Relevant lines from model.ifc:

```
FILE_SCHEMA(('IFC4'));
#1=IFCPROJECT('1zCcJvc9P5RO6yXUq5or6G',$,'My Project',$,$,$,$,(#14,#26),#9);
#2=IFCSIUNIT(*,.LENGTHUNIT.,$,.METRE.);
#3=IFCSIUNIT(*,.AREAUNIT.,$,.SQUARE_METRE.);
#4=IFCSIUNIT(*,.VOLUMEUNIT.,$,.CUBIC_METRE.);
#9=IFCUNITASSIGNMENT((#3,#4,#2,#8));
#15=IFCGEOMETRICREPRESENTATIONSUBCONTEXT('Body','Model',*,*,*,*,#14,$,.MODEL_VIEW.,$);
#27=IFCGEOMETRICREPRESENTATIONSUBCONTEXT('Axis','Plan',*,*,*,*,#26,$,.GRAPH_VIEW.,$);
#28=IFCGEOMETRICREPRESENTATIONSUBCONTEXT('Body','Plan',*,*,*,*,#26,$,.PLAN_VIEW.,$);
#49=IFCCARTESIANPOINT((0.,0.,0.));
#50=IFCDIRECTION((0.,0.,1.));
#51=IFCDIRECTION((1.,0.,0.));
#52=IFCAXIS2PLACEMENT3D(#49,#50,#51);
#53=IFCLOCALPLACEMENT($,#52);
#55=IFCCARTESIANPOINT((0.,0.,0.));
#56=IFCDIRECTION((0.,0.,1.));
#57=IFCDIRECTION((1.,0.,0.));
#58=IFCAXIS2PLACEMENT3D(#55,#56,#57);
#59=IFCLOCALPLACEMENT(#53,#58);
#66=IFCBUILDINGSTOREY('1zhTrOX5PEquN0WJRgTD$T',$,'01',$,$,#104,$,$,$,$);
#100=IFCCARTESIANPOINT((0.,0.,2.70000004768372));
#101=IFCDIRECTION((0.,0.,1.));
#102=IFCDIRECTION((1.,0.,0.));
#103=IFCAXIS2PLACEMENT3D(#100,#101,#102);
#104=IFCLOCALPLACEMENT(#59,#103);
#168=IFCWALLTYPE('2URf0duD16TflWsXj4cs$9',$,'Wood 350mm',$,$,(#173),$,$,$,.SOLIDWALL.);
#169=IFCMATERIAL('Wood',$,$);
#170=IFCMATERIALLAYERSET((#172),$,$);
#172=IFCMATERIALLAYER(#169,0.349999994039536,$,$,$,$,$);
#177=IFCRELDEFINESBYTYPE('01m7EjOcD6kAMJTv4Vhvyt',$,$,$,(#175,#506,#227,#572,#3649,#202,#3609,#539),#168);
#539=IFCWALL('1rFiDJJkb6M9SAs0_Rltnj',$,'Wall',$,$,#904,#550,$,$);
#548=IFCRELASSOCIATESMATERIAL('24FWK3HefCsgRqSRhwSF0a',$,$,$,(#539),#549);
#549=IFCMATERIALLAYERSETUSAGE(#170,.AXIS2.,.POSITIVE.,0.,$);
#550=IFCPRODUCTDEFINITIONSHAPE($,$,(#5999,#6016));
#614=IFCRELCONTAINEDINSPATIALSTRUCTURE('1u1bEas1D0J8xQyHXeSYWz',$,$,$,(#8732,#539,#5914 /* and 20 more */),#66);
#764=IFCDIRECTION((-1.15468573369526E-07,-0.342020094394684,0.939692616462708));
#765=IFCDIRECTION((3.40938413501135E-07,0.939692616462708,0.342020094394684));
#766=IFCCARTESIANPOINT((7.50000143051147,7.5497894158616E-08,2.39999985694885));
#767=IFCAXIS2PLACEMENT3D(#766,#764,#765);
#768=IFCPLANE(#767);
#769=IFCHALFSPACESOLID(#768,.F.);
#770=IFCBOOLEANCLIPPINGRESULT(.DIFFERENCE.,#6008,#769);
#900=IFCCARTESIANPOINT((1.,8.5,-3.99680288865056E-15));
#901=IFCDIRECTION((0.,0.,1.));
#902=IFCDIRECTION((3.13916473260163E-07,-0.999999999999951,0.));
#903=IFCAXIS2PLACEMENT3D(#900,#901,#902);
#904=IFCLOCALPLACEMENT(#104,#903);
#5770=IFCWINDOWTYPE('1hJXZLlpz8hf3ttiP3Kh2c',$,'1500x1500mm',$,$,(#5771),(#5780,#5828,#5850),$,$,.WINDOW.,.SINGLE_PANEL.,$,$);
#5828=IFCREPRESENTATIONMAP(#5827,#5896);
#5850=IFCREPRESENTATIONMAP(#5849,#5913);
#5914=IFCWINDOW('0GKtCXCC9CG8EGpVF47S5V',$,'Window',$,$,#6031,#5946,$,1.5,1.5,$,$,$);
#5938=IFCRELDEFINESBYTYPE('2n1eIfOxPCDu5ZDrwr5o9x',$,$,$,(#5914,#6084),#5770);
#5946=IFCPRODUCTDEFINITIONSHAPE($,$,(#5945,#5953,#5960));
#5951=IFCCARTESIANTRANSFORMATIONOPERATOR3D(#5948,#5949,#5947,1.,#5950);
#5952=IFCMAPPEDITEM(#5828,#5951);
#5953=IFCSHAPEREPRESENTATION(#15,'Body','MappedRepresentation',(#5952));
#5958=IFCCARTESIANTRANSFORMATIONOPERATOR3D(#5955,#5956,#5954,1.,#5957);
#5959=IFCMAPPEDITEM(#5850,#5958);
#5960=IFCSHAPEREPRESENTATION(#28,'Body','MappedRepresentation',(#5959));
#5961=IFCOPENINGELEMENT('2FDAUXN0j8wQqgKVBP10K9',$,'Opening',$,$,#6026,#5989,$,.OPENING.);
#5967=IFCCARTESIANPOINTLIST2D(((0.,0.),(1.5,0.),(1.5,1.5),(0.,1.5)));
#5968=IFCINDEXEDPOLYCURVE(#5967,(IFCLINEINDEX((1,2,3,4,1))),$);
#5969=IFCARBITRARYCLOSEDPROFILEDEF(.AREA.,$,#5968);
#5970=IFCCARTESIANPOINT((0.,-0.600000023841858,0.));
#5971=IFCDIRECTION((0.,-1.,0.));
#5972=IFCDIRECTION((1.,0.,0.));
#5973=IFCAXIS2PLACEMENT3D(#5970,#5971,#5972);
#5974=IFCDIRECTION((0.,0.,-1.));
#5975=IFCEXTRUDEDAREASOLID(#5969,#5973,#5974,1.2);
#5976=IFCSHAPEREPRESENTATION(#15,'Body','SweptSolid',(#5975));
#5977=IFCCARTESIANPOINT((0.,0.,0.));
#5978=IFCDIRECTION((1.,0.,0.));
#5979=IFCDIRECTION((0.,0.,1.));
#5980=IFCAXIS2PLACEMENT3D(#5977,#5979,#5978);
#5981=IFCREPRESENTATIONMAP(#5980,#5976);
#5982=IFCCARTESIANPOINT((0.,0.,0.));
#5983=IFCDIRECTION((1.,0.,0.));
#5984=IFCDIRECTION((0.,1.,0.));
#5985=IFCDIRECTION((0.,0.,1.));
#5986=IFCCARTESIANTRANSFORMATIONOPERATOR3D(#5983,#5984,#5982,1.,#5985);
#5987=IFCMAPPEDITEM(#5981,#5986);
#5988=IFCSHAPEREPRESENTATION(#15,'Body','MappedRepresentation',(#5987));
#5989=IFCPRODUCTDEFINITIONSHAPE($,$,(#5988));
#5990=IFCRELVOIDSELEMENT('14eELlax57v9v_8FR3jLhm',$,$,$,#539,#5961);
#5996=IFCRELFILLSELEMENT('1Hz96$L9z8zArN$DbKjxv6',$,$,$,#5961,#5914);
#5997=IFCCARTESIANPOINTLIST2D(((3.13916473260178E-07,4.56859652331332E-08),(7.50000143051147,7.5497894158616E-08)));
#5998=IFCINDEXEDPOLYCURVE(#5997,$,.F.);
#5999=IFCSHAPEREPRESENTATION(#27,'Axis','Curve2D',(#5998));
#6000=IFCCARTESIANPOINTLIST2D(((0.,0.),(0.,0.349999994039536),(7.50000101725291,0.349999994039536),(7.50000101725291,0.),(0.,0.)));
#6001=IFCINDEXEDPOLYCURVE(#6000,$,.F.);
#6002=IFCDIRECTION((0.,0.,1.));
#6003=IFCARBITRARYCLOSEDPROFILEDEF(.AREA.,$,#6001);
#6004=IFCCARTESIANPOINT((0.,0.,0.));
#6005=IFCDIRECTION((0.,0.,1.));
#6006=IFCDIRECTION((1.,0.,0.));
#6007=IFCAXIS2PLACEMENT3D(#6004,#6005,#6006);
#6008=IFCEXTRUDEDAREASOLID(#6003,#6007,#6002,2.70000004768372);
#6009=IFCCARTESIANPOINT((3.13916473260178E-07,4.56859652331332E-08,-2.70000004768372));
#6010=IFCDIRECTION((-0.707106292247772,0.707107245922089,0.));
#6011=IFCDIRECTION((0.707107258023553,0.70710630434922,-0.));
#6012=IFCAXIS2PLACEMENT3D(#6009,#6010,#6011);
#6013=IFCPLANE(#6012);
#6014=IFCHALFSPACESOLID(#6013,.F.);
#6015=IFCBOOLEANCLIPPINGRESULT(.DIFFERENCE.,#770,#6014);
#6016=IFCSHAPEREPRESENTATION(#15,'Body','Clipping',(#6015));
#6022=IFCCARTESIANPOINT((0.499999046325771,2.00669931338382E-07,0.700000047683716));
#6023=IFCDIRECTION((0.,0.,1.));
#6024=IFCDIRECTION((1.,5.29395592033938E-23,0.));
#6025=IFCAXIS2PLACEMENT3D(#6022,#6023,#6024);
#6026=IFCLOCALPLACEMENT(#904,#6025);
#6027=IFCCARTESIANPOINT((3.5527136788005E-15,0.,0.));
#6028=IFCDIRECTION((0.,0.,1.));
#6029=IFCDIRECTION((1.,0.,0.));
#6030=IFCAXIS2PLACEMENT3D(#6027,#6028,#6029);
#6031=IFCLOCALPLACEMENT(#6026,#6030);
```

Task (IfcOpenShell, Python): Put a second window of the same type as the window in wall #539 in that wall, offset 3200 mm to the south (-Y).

```python
import ifcopenshell
import ifcopenshell.api.feature
import ifcopenshell.api.geometry
import ifcopenshell.api.root
import ifcopenshell.geom
import ifcopenshell.util.element
import ifcopenshell.util.placement
import ifcopenshell.util.shape

model = ifcopenshell.open("model.ifc")
settings = ifcopenshell.geom.settings()


def volume(element):
    """Net volume in cubic metres, openings subtracted."""
    shape = ifcopenshell.geom.create_shape(settings, element)
    return ifcopenshell.util.shape.get_volume(shape.geometry)


window = model.by_guid("0GKtCXCC9CG8EGpVF47S5V")
opening = window.FillsVoids[0].RelatingOpeningElement
wall = opening.VoidsElements[0].RelatingBuildingElement
before = volume(wall)
shift = ifcopenshell.util.placement.get_local_placement(wall.ObjectPlacement)[:3, 0] * 3.2

# copy_class copies the void relationship, type, container and properties, but no geometry.
new_opening = ifcopenshell.api.root.copy_class(model, product=opening)
new_opening.Representation = ifcopenshell.util.element.copy_deep(
    model, opening.Representation, exclude=["IfcGeometricRepresentationContext", "IfcRepresentationMap"]
)
new_window = ifcopenshell.api.root.copy_class(model, product=window)
new_window.Representation = ifcopenshell.util.element.copy_deep(
    model, window.Representation, exclude=["IfcGeometricRepresentationContext", "IfcRepresentationMap"]
)
ifcopenshell.api.feature.add_filling(model, opening=new_opening, element=new_window)

for old, new in ((opening, new_opening), (window, new_window)):
    matrix = ifcopenshell.util.placement.get_local_placement(old.ObjectPlacement)
    matrix[:3, 3] += shift
    ifcopenshell.api.geometry.edit_object_placement(model, product=new, matrix=matrix, is_si=False)

after = volume(wall)

print(f"wall volume {before:.3f} -> {after:.3f} m3")

model.write("model_updated.ifc")
```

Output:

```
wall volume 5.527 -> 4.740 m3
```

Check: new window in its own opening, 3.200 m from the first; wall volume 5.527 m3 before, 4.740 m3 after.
